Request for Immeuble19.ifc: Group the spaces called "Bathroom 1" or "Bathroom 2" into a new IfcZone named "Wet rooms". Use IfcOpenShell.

First a look at what the model holds.

```python
import ifcopenshell

model = ifcopenshell.open("Immeuble19.ifc")
print(model.schema)
seen = {}
for space in model.by_type("IfcSpace"):
    seen[space.LongName] = seen.get(space.LongName, 0) + 1
for name, count in sorted(seen.items(), key=str):
    print(count, "x", name)
print("zones:", [z.Name for z in model.by_type("IfcZone")][:20])
```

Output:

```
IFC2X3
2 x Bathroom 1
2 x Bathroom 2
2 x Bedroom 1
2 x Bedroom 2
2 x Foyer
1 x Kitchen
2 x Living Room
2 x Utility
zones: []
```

```python
import ifcopenshell
import ifcopenshell.api.group
import ifcopenshell.api.root

model = ifcopenshell.open("Immeuble19.ifc")

names = {"Bathroom 1", "Bathroom 2"}
spaces = [s for s in model.by_type("IfcSpace") if s.LongName in names]

zone = ifcopenshell.api.root.create_entity(model, ifc_class="IfcZone", name="Wet rooms")
ifcopenshell.api.group.assign_group(model, products=spaces, group=zone)
print(len(spaces), "spaces in", zone.Name)

model.write("Immeuble19_edited.ifc")
```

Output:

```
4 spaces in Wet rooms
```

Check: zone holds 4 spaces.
